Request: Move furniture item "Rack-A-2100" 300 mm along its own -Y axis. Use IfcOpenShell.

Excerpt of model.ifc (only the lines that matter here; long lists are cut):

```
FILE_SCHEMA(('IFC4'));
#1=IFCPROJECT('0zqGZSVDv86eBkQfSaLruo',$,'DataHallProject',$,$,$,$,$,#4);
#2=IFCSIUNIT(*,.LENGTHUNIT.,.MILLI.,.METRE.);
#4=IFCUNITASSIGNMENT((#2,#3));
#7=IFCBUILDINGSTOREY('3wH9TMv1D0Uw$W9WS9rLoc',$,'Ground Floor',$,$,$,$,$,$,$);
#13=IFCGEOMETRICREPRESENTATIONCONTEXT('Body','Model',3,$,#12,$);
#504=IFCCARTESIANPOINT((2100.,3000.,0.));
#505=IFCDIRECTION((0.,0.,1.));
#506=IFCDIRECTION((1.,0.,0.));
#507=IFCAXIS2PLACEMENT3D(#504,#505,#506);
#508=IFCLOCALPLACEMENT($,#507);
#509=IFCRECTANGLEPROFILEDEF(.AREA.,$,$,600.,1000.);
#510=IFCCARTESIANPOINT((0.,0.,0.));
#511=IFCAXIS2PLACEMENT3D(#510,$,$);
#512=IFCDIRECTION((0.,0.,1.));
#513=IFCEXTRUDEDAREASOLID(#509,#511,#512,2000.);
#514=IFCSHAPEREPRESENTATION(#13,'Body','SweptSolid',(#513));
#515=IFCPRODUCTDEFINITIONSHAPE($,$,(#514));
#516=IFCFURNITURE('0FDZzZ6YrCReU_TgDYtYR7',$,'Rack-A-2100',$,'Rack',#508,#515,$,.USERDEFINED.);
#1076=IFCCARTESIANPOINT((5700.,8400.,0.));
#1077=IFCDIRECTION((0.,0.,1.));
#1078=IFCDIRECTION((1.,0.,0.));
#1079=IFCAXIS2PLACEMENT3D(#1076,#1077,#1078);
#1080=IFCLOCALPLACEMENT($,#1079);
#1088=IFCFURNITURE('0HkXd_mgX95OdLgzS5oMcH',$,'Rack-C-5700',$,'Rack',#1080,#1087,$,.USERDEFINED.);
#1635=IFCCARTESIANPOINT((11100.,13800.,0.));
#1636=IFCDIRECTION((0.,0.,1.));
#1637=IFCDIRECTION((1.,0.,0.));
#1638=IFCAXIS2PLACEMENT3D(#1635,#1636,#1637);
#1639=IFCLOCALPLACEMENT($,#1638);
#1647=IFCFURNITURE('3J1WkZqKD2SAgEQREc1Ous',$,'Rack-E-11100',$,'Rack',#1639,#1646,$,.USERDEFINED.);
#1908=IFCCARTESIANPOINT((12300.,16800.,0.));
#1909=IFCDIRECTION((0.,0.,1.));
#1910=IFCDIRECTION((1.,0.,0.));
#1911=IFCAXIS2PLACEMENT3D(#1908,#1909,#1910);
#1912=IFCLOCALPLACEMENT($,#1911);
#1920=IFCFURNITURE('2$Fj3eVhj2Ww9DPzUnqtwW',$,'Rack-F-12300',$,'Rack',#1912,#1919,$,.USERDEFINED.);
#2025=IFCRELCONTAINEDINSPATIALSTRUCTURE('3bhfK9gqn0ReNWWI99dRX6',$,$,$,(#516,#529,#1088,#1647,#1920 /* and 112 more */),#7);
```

```python
import ifcopenshell
import ifcopenshell.api.geometry
import ifcopenshell.util.placement

model = ifcopenshell.open("model.ifc")

item = model.by_guid("0FDZzZ6YrCReU_TgDYtYR7")
matrix = ifcopenshell.util.placement.get_local_placement(item.ObjectPlacement)
matrix[:3, 3] -= matrix[:3, 1] * 300.0
ifcopenshell.api.geometry.edit_object_placement(model, product=item, matrix=matrix, is_si=False)

print(ifcopenshell.util.placement.get_local_placement(item.ObjectPlacement).round(3) + 0.0)

model.write("model-out.ifc")
```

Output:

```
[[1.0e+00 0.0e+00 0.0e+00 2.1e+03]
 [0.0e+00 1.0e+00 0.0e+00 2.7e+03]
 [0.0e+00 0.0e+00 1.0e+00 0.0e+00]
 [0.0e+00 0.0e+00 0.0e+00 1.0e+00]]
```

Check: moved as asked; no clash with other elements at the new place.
